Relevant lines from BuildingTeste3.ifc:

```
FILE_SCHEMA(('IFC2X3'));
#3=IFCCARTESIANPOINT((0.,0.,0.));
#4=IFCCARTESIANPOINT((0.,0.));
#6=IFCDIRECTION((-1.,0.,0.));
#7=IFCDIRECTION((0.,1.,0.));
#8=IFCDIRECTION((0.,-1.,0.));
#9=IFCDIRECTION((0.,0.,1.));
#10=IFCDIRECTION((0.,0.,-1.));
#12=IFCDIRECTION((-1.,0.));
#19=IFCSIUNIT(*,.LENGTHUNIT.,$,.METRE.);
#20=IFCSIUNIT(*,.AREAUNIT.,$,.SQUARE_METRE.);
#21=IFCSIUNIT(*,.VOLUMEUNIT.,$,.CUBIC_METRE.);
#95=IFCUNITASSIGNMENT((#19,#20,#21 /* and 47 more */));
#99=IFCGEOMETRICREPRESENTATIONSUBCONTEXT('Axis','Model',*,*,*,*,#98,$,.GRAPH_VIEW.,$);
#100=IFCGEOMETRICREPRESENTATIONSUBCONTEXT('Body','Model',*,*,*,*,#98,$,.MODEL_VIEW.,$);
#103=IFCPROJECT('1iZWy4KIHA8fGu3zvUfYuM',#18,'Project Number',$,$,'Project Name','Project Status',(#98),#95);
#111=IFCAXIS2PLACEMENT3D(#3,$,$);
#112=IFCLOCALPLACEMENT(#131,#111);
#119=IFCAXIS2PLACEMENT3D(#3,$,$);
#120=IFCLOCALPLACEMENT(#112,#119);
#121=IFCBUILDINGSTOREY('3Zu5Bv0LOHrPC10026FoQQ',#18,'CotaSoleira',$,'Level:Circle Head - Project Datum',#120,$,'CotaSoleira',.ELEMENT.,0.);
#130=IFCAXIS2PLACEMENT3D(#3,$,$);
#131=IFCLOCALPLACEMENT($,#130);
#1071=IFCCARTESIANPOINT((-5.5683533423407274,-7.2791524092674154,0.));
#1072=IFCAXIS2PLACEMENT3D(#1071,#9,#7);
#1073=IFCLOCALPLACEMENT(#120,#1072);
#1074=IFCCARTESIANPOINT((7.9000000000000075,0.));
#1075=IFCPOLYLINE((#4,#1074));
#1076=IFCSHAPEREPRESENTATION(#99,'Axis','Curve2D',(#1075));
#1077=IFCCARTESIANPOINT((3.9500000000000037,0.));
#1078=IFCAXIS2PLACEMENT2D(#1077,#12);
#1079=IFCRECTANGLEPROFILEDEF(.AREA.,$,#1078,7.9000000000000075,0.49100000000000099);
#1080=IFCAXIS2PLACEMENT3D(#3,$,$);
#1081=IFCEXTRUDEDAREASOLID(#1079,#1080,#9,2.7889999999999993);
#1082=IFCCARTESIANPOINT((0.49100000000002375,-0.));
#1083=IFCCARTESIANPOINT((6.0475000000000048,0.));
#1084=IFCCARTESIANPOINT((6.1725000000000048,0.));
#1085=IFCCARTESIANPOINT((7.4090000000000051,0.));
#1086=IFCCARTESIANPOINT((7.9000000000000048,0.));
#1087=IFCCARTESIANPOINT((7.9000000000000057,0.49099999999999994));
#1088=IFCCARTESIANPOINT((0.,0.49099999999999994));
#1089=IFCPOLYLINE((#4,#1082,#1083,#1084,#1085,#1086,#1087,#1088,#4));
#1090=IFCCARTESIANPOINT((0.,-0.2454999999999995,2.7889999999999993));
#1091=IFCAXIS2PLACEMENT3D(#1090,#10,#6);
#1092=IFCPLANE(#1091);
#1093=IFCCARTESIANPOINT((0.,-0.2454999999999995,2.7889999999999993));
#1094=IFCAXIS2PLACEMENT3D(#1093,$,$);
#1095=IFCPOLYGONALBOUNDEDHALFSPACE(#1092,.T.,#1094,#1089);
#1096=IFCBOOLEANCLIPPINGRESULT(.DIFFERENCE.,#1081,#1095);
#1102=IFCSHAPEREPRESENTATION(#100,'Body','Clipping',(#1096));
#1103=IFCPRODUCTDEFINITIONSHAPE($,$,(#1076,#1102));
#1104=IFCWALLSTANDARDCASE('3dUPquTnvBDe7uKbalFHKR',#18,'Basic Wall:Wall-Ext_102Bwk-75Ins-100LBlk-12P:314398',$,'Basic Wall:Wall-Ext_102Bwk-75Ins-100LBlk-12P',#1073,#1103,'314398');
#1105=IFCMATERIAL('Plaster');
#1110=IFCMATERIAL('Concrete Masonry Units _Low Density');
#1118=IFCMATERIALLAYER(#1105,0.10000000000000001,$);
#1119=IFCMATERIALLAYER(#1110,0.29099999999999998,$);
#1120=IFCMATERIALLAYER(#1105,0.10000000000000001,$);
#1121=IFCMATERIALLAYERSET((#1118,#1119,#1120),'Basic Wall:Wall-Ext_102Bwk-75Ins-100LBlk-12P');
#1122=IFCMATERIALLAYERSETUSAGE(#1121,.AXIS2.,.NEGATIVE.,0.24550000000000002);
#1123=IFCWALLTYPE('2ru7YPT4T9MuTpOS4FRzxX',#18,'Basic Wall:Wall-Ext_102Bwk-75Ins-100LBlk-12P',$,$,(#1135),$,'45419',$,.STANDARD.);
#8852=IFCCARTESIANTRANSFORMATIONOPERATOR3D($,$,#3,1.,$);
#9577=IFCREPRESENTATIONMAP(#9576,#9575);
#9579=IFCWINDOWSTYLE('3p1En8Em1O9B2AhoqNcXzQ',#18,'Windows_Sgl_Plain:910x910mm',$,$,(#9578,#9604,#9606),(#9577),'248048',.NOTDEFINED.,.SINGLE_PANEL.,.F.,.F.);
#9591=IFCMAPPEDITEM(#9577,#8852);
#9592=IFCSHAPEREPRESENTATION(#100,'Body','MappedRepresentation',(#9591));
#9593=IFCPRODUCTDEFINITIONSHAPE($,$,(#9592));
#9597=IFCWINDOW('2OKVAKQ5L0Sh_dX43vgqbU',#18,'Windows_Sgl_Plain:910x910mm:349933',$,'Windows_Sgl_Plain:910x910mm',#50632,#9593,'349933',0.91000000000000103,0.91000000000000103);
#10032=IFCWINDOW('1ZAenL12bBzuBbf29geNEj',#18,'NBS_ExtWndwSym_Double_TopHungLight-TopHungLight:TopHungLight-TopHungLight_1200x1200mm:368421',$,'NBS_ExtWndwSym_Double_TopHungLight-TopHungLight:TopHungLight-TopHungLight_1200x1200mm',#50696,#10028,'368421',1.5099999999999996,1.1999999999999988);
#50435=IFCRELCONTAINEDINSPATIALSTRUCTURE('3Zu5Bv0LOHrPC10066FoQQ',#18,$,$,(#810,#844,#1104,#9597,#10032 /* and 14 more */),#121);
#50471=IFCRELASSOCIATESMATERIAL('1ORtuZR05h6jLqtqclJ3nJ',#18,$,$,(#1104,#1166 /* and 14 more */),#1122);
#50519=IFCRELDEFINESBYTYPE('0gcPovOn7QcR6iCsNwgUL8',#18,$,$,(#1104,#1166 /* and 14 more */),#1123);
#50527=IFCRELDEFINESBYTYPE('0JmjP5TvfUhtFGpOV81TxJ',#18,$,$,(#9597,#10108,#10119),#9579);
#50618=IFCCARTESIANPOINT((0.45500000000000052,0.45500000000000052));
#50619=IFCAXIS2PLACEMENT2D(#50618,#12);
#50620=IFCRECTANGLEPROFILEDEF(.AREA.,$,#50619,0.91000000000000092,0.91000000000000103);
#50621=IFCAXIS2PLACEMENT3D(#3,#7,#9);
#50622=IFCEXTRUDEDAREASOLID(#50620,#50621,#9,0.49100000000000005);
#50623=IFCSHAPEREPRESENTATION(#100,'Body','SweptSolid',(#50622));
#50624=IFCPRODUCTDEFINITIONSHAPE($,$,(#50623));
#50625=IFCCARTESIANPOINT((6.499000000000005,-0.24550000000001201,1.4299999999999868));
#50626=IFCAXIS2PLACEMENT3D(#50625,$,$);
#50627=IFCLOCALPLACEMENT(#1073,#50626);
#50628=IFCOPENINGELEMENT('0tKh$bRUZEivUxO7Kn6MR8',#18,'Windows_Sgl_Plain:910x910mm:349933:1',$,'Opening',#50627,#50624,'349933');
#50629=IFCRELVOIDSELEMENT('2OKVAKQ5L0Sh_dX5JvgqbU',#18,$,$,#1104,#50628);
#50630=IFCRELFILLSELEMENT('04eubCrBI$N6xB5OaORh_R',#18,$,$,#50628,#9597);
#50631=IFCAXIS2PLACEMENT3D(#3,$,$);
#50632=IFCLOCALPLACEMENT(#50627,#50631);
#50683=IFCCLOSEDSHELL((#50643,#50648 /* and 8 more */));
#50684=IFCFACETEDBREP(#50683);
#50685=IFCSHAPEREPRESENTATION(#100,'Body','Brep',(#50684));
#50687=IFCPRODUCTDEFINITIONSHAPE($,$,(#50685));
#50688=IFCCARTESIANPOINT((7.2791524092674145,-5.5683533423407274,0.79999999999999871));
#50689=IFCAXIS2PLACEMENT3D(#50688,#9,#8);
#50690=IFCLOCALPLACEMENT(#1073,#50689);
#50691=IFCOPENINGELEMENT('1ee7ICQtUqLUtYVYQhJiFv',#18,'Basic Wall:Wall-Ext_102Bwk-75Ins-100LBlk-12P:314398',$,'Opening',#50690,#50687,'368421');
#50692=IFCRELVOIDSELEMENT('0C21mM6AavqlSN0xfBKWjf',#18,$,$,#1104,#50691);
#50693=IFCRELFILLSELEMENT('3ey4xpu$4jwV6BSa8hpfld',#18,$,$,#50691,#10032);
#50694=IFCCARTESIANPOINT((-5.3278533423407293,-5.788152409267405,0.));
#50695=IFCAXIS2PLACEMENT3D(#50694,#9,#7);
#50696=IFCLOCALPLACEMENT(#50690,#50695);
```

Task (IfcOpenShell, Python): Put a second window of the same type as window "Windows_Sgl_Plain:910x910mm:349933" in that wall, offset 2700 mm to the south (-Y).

```python
import ifcopenshell
import ifcopenshell.api.feature
import ifcopenshell.api.geometry
import ifcopenshell.api.root
import ifcopenshell.geom
import ifcopenshell.util.element
import ifcopenshell.util.placement
import ifcopenshell.util.shape
import ifcopenshell.util.unit

model = ifcopenshell.open("BuildingTeste3.ifc")
unit_scale = ifcopenshell.util.unit.calculate_unit_scale(model)
settings = ifcopenshell.geom.settings()


def volume(element):
    """Net volume in cubic metres, openings subtracted."""
    shape = ifcopenshell.geom.create_shape(settings, element)
    return ifcopenshell.util.shape.get_volume(shape.geometry)


def reuse_history(source, copy):
    """copy_class also copies each property set's owner history, people and application; keep the originals."""
    for rel in copy.IsDefinedBy:
        if rel.is_a("IfcRelDefinesByProperties") and (history := rel.RelatingPropertyDefinition.OwnerHistory):
            rel.RelatingPropertyDefinition.OwnerHistory = source.OwnerHistory
            ifcopenshell.util.element.remove_deep2(model, history)


window = model.by_id(9597)
opening = window.FillsVoids[0].RelatingOpeningElement
wall = opening.VoidsElements[0].RelatingBuildingElement
before = volume(wall)
shift = ifcopenshell.util.placement.get_local_placement(wall.ObjectPlacement)[:3, 0] * -2.7 / unit_scale

# copy_class copies the void relationship, type, container and properties, but no geometry.
new_opening = ifcopenshell.api.root.copy_class(model, product=opening)
new_opening.Representation = ifcopenshell.util.element.copy_deep(
    model, opening.Representation, exclude=["IfcGeometricRepresentationContext", "IfcRepresentationMap"]
)
new_opening.Name = "Windows_Sgl_Plain:910x910mm"
new_opening.Tag = None
new_window = ifcopenshell.api.root.copy_class(model, product=window)
new_window.Representation = ifcopenshell.util.element.copy_deep(
    model, window.Representation, exclude=["IfcGeometricRepresentationContext", "IfcRepresentationMap"]
)
new_window.Name = "Windows_Sgl_Plain:910x910mm"
new_window.Tag = None
reuse_history(window, new_window)
fills = ifcopenshell.api.feature.add_filling(model, opening=new_opening, element=new_window)
fills.OwnerHistory = new_window.OwnerHistory  # required in IFC2X3

for old, new in ((opening, new_opening), (window, new_window)):
    matrix = ifcopenshell.util.placement.get_local_placement(old.ObjectPlacement)
    matrix[:3, 3] += shift
    ifcopenshell.api.geometry.edit_object_placement(model, product=new, matrix=matrix, is_si=False)

after = volume(wall)

print(f"wall volume {before:.3f} -> {after:.3f} m3")

model.write("BuildingTeste3_v2.ifc")
```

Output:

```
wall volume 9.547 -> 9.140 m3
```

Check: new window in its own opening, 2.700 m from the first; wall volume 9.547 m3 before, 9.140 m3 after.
